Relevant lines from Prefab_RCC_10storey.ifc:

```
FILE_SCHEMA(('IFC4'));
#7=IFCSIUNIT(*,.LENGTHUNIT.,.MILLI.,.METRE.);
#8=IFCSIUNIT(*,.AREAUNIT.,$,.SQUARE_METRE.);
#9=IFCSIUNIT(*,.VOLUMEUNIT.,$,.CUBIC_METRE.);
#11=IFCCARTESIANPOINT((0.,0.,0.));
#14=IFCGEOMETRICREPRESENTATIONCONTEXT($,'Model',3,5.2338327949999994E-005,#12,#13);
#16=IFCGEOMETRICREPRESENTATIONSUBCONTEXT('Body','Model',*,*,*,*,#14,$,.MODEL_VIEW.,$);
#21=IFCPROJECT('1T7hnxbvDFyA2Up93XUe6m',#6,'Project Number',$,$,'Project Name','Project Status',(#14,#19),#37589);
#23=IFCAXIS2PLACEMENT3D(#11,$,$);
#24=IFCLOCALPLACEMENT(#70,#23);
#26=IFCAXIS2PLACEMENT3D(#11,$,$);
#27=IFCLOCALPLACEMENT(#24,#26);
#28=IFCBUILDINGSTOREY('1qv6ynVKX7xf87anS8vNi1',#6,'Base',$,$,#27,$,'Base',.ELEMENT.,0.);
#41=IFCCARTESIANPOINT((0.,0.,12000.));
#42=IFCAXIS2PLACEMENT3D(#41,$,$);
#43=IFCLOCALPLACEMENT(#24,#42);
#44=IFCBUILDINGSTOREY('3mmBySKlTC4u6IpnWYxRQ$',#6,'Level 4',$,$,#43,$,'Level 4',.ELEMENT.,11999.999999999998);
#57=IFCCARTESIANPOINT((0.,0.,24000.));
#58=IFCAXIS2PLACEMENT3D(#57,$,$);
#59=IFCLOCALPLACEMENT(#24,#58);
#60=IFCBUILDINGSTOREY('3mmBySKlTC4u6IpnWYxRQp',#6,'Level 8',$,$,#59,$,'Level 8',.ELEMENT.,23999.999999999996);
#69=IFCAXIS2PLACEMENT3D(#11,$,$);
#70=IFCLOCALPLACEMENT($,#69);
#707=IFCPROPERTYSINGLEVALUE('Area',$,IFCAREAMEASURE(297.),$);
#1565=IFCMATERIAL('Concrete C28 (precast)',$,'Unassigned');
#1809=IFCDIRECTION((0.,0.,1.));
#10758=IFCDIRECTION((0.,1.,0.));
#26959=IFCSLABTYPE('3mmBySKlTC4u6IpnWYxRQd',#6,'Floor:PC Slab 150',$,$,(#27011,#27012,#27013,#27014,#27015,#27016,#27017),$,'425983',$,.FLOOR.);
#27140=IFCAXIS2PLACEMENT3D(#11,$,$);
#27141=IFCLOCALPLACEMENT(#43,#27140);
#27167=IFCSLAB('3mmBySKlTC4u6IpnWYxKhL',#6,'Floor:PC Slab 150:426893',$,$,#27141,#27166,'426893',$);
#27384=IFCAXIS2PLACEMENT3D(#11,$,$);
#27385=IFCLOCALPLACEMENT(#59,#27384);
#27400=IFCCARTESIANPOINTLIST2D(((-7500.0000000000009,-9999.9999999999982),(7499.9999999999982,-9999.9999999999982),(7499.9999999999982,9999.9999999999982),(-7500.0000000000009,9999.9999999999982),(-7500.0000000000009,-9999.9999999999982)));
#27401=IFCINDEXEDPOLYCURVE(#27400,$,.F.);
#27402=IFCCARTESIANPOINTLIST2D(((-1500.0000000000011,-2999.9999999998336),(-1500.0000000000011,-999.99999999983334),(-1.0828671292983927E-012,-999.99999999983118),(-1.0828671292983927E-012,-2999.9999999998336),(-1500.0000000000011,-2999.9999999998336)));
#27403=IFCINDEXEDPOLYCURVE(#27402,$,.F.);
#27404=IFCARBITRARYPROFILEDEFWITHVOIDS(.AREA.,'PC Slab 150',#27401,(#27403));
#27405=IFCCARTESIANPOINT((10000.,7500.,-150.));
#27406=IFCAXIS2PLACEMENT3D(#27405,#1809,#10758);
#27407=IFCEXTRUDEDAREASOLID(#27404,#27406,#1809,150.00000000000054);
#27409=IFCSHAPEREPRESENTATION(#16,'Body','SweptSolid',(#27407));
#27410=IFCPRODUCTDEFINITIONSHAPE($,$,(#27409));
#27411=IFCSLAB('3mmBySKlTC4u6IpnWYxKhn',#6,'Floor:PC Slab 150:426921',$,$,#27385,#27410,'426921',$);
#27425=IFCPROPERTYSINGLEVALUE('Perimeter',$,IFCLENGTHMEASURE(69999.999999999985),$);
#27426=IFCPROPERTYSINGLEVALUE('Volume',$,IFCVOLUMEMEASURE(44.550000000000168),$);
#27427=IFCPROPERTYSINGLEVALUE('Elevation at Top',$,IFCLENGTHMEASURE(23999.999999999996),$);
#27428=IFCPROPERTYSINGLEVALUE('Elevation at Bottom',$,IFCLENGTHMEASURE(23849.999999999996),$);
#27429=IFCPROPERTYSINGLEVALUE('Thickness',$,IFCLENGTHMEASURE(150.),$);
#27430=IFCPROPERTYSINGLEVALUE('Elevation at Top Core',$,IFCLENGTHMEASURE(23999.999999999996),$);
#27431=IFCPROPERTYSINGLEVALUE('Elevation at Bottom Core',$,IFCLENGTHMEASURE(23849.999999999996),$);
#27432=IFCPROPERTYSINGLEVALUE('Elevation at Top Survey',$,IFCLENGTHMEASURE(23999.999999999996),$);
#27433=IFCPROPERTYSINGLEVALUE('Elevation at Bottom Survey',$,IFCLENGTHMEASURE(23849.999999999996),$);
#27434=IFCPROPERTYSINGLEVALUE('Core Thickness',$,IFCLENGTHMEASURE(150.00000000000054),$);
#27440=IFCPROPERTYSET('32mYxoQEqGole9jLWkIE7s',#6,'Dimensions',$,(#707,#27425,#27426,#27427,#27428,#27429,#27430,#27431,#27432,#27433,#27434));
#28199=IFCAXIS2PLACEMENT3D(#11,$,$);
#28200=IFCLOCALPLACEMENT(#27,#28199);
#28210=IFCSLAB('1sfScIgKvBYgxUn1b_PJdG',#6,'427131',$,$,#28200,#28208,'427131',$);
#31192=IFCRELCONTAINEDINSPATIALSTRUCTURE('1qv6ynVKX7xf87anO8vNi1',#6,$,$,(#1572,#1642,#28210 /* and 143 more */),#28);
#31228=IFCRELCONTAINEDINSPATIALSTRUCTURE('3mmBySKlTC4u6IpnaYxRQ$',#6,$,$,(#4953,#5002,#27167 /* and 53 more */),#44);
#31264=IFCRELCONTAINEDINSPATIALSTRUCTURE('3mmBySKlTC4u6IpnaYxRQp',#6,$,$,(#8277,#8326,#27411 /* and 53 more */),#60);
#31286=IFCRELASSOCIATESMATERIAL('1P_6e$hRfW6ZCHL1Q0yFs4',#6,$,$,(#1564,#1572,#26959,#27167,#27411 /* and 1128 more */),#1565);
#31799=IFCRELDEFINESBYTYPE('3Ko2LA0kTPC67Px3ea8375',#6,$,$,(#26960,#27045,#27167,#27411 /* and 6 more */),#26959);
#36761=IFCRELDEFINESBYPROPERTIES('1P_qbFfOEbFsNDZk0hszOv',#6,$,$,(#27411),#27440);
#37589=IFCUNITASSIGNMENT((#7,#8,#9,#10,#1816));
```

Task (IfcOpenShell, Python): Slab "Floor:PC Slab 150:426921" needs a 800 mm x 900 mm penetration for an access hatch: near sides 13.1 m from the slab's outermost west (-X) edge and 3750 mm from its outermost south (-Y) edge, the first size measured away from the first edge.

```python
import numpy as np
import ifcopenshell
import ifcopenshell.api.feature
import ifcopenshell.api.geometry
import ifcopenshell.api.pset
import ifcopenshell.api.root
import ifcopenshell.geom
import ifcopenshell.util.element
import ifcopenshell.util.placement
import ifcopenshell.util.representation
import ifcopenshell.util.shape
import ifcopenshell.util.unit

model = ifcopenshell.open("Prefab_RCC_10storey.ifc")
unit_scale = ifcopenshell.util.unit.calculate_unit_scale(model)
area_scale = ifcopenshell.util.unit.calculate_unit_scale(model, "AREAUNIT")
volume_scale = ifcopenshell.util.unit.calculate_unit_scale(model, "VOLUMEUNIT")
settings = ifcopenshell.geom.settings()


def volume(element):
    """Net volume in cubic metres, openings subtracted."""
    shape = ifcopenshell.geom.create_shape(settings, element)
    return ifcopenshell.util.shape.get_volume(shape.geometry)


slab = model.by_id(27411)
before = volume(slab)

# Extent in the slab's own axes, in metres. The edges named are its -X and -Y sides.
slab_shape = ifcopenshell.geom.create_shape(settings, slab)
vertices = ifcopenshell.util.shape.get_vertices(slab_shape.geometry)
x_min, y_min, bottom = vertices.min(axis=0)
top = vertices[:, 2].max()

opening = ifcopenshell.api.root.create_entity(model, ifc_class="IfcOpeningElement", name="Access hatch opening", predefined_type="OPENING")
context = ifcopenshell.util.representation.get_context(model, "Model", "Body", "MODEL_VIEW")
width, depth = 0.8, 0.9
outline = [(0.0, 0.0), (width, 0.0), (width, depth), (0.0, depth), (0.0, 0.0)]
# Overshoot both faces by 50 mm so the cut is clean.
shape = ifcopenshell.api.geometry.add_slab_representation(
    model, context=context, depth=top - bottom + 0.1, polyline=outline
)
ifcopenshell.api.geometry.assign_representation(model, product=opening, representation=shape)

matrix = ifcopenshell.util.placement.get_local_placement(slab.ObjectPlacement)
matrix[:, 3] = matrix @ np.append(np.array([x_min + 13.1, y_min + 3.75, bottom - 0.05]) / unit_scale, 1.0)
ifcopenshell.api.geometry.edit_object_placement(model, product=opening, matrix=matrix, is_si=False)
ifcopenshell.api.feature.add_feature(model, feature=opening, element=slab)

after = volume(slab)

# Update the slab's stored quantities.
pset = model.by_id(ifcopenshell.util.element.get_pset(slab, "Dimensions", should_inherit=False)["id"])
ifcopenshell.api.pset.edit_pset(model, pset=pset, properties={
    "Area": model.create_entity("IfcAreaMeasure", after / (top - bottom) / area_scale),
    "Volume": model.create_entity("IfcVolumeMeasure", after / volume_scale),
})

print(f"slab volume {before:.3f} -> {after:.3f} m3")

model.write("Prefab_RCC_10storey_updated.ifc")
```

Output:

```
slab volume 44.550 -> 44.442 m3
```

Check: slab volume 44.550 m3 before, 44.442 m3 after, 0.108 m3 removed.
